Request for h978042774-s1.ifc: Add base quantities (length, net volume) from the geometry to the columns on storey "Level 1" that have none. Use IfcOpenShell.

First a look at what the model holds.

```python
import ifcopenshell
import ifcopenshell.util.element
import ifcopenshell.util.unit

model = ifcopenshell.open("h978042774-s1.ifc")
print(model.schema)
for unit_type in ("LENGTHUNIT", "AREAUNIT", "VOLUMEUNIT"):
    print(unit_type, ifcopenshell.util.unit.calculate_unit_scale(model, unit_type))
storey = next(s for s in model.by_type("IfcBuildingStorey") if s.Name == "Level 1")
columns = [e for e in ifcopenshell.util.element.get_decomposition(storey) if e.is_a("IfcColumn")]
for e in sorted(columns, key=lambda e: e.id()):
    print(e.id(), e.is_a(), e.Name, list(ifcopenshell.util.element.get_psets(e, qtos_only=True)), sep=" | ")
```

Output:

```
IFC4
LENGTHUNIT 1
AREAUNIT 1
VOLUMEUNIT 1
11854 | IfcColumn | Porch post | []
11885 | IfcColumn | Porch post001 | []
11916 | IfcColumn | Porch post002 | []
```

```python
import ifcopenshell
import ifcopenshell.api.pset
import ifcopenshell.geom
import ifcopenshell.util.element
import ifcopenshell.util.shape
import ifcopenshell.util.unit

model = ifcopenshell.open("h978042774-s1.ifc")
unit_scale = ifcopenshell.util.unit.calculate_unit_scale(model)
volume_scale = ifcopenshell.util.unit.calculate_unit_scale(model, "VOLUMEUNIT")
settings = ifcopenshell.geom.settings()

storey = next(s for s in model.by_type("IfcBuildingStorey") if s.Name == "Level 1")
columns = [e for e in ifcopenshell.util.element.get_decomposition(storey) if e.is_a("IfcColumn")]

for e in sorted(columns, key=lambda e: e.id()):
    if ifcopenshell.util.element.get_psets(e, qtos_only=True, should_inherit=False):
        continue
    # Geometry comes back in metres, in the element's own axes.
    shape = ifcopenshell.geom.create_shape(settings, e)
    values = {
        "Length": ifcopenshell.util.shape.get_z(shape.geometry) / unit_scale,
        "NetVolume": ifcopenshell.util.shape.get_volume(shape.geometry) / volume_scale,
    }
    qto = ifcopenshell.api.pset.add_qto(model, product=e, name="Qto_ColumnBaseQuantities")
    ifcopenshell.api.pset.edit_qto(model, qto=qto, properties=values)
    print(e.id(), {k: round(v, 3) for k, v in values.items()})

model.write("h978042774-s1_edited.ifc")
```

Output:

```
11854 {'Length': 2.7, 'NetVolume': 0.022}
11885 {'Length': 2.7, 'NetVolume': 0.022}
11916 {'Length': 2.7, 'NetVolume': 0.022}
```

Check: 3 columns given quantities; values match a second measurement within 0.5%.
